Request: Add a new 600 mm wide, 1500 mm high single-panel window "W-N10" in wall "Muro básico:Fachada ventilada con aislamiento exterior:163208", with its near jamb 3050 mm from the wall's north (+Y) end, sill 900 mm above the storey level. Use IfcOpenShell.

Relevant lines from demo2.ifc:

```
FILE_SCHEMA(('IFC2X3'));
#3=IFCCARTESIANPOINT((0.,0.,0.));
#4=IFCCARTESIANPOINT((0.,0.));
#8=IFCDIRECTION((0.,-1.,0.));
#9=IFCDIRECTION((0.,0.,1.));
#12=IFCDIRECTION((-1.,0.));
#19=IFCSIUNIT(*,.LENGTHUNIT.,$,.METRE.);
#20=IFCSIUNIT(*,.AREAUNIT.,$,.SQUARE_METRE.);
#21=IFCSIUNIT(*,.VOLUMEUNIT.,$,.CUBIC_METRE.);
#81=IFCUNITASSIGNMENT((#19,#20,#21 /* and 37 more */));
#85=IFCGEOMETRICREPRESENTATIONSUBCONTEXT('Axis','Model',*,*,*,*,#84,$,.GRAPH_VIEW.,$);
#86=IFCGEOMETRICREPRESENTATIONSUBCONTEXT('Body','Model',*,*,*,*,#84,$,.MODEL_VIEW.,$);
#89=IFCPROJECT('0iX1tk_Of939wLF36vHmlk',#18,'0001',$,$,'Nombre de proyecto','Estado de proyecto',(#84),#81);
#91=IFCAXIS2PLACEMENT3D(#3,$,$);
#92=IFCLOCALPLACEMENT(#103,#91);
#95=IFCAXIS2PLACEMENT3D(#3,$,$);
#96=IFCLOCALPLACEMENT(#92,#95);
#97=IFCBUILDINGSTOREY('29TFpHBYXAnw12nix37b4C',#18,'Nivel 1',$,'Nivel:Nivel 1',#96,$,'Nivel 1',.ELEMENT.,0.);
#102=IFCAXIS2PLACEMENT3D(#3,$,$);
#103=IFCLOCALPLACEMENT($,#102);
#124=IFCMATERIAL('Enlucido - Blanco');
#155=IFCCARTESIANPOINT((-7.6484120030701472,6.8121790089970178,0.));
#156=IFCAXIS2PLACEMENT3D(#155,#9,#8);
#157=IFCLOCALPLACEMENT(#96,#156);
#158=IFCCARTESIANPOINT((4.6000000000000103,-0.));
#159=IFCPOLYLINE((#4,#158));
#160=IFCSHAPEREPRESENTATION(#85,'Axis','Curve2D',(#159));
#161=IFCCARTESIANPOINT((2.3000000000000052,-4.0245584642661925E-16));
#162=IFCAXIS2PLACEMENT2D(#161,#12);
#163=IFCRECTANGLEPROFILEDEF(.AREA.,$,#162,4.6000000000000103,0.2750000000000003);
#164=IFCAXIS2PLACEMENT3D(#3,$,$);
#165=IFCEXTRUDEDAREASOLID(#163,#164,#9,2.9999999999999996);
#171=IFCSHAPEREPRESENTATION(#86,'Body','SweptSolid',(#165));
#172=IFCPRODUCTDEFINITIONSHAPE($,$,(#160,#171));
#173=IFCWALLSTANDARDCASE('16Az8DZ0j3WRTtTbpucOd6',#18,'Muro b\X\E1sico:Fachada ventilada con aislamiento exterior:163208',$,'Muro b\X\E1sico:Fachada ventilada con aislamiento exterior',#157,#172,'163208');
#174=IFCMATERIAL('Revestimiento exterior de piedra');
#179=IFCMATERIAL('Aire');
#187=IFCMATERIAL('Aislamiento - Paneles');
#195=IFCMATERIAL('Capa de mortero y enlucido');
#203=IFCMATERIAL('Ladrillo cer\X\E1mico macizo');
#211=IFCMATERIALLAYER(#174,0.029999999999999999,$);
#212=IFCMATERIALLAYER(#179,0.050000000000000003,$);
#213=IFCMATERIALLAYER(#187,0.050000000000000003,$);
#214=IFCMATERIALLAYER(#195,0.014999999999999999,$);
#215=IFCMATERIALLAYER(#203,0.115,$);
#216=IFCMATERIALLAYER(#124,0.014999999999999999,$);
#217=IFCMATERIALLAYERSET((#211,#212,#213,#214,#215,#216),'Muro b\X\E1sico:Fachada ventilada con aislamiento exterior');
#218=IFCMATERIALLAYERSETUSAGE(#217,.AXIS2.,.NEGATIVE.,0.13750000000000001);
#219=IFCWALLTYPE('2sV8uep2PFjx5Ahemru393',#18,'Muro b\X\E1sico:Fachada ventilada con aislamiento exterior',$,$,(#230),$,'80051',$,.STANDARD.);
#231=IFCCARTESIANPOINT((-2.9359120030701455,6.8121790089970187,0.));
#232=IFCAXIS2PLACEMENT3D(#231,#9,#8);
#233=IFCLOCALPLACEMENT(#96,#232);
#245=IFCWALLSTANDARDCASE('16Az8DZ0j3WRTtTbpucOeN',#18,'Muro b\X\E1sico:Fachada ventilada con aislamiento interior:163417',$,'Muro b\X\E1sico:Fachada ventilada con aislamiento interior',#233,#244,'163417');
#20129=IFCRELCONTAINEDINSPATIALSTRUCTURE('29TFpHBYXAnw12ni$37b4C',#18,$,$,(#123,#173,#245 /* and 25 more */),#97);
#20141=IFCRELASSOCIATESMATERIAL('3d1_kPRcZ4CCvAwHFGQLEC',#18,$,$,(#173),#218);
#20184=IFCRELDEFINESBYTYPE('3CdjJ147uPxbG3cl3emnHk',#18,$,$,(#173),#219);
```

```python
import numpy as np
import ifcopenshell
import ifcopenshell.api.feature
import ifcopenshell.api.geometry
import ifcopenshell.api.root
import ifcopenshell.api.spatial
import ifcopenshell.api.type
import ifcopenshell.geom
import ifcopenshell.util.element
import ifcopenshell.util.placement
import ifcopenshell.util.representation
import ifcopenshell.util.shape
import ifcopenshell.util.unit

model = ifcopenshell.open("demo2.ifc")
unit_scale = ifcopenshell.util.unit.calculate_unit_scale(model)
settings = ifcopenshell.geom.settings()


def volume(element):
    """Net volume in cubic metres, openings subtracted."""
    shape = ifcopenshell.geom.create_shape(settings, element)
    return ifcopenshell.util.shape.get_volume(shape.geometry)


wall = model.by_guid("16Az8DZ0j3WRTtTbpucOd6")
storey = ifcopenshell.util.element.get_container(wall, ifc_class="IfcBuildingStorey")
context = ifcopenshell.util.representation.get_context(model, "Model", "Body", "MODEL_VIEW")
before = volume(wall)

width, height, from_end, sill = 0.6, 1.5, 3.05, 0.9  # metres

# The wall runs along its own X axis, and the end named is its -X end.
wall_shape = ifcopenshell.geom.create_shape(settings, wall)
x, y, z = ifcopenshell.util.shape.get_vertices(wall_shape.geometry).T
start = x.min() + from_end
face, thickness = float(y.min()), float(y.max() - y.min())
wall_matrix = ifcopenshell.util.placement.get_local_placement(wall.ObjectPlacement)
level = ifcopenshell.util.placement.get_local_placement(storey.ObjectPlacement)[2, 3]


def in_wall(x, y):
    """Placement at x, y metres in the wall's axes, at sill height."""
    matrix = wall_matrix.copy()
    matrix[:, 3] = wall_matrix @ np.array([x / unit_scale, y / unit_scale, 0.0, 1.0])
    matrix[2, 3] = level + sill / unit_scale
    return matrix


# Opening: a box that overshoots both wall faces by 50 mm.
opening = ifcopenshell.api.root.create_entity(model, ifc_class="IfcOpeningElement")
box = ifcopenshell.api.geometry.add_wall_representation(
    model, context=context, length=width, height=height, thickness=thickness + 0.1
)
ifcopenshell.api.geometry.assign_representation(model, product=opening, representation=box)
ifcopenshell.api.geometry.edit_object_placement(model, product=opening, matrix=in_wall(start, face - 0.05), is_si=False)
ifcopenshell.api.feature.add_feature(model, feature=opening, element=wall)

window = ifcopenshell.api.root.create_entity(model, ifc_class="IfcWindow", name="W-N10")
window.OverallWidth, window.OverallHeight = width / unit_scale, height / unit_scale
body = ifcopenshell.api.geometry.add_window_representation(
    model,
    context=context,
    overall_width=window.OverallWidth,
    overall_height=window.OverallHeight,
    partition_type="SINGLE_PANEL",
)
ifcopenshell.api.geometry.assign_representation(model, product=window, representation=body)
ifcopenshell.api.spatial.assign_container(model, products=[window], relating_structure=storey)
fills = ifcopenshell.api.feature.add_filling(model, opening=opening, element=window)
fills.OwnerHistory = window.OwnerHistory  # required in IFC2X3

# IFC2X3 keeps the operation on the window style.
style = ifcopenshell.api.root.create_entity(model, ifc_class="IfcWindowStyle", name="W-N10")
style.OperationType, style.ConstructionType = "SINGLE_PANEL", "NOTDEFINED"
style.ParameterTakesPrecedence = style.Sizeable = False
ifcopenshell.api.type.assign_type(model, related_objects=[window], relating_type=style)

# Centre the window in the wall's thickness.
ifcopenshell.api.geometry.edit_object_placement(model, product=window, matrix=in_wall(start, face), is_si=False)
window_shape = ifcopenshell.geom.create_shape(settings, window)
depth = ifcopenshell.util.shape.get_vertices(window_shape.geometry)[:, 1]
offset = face + thickness / 2 - (depth.min() + depth.max()) / 2
ifcopenshell.api.geometry.edit_object_placement(model, product=window, matrix=in_wall(start, offset), is_si=False)

after = volume(wall)

print(f"wall volume {before:.3f} -> {after:.3f} m3")

model.write("demo2-out.ifc")
```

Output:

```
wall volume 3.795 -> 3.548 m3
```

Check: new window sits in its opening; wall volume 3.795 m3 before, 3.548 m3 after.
